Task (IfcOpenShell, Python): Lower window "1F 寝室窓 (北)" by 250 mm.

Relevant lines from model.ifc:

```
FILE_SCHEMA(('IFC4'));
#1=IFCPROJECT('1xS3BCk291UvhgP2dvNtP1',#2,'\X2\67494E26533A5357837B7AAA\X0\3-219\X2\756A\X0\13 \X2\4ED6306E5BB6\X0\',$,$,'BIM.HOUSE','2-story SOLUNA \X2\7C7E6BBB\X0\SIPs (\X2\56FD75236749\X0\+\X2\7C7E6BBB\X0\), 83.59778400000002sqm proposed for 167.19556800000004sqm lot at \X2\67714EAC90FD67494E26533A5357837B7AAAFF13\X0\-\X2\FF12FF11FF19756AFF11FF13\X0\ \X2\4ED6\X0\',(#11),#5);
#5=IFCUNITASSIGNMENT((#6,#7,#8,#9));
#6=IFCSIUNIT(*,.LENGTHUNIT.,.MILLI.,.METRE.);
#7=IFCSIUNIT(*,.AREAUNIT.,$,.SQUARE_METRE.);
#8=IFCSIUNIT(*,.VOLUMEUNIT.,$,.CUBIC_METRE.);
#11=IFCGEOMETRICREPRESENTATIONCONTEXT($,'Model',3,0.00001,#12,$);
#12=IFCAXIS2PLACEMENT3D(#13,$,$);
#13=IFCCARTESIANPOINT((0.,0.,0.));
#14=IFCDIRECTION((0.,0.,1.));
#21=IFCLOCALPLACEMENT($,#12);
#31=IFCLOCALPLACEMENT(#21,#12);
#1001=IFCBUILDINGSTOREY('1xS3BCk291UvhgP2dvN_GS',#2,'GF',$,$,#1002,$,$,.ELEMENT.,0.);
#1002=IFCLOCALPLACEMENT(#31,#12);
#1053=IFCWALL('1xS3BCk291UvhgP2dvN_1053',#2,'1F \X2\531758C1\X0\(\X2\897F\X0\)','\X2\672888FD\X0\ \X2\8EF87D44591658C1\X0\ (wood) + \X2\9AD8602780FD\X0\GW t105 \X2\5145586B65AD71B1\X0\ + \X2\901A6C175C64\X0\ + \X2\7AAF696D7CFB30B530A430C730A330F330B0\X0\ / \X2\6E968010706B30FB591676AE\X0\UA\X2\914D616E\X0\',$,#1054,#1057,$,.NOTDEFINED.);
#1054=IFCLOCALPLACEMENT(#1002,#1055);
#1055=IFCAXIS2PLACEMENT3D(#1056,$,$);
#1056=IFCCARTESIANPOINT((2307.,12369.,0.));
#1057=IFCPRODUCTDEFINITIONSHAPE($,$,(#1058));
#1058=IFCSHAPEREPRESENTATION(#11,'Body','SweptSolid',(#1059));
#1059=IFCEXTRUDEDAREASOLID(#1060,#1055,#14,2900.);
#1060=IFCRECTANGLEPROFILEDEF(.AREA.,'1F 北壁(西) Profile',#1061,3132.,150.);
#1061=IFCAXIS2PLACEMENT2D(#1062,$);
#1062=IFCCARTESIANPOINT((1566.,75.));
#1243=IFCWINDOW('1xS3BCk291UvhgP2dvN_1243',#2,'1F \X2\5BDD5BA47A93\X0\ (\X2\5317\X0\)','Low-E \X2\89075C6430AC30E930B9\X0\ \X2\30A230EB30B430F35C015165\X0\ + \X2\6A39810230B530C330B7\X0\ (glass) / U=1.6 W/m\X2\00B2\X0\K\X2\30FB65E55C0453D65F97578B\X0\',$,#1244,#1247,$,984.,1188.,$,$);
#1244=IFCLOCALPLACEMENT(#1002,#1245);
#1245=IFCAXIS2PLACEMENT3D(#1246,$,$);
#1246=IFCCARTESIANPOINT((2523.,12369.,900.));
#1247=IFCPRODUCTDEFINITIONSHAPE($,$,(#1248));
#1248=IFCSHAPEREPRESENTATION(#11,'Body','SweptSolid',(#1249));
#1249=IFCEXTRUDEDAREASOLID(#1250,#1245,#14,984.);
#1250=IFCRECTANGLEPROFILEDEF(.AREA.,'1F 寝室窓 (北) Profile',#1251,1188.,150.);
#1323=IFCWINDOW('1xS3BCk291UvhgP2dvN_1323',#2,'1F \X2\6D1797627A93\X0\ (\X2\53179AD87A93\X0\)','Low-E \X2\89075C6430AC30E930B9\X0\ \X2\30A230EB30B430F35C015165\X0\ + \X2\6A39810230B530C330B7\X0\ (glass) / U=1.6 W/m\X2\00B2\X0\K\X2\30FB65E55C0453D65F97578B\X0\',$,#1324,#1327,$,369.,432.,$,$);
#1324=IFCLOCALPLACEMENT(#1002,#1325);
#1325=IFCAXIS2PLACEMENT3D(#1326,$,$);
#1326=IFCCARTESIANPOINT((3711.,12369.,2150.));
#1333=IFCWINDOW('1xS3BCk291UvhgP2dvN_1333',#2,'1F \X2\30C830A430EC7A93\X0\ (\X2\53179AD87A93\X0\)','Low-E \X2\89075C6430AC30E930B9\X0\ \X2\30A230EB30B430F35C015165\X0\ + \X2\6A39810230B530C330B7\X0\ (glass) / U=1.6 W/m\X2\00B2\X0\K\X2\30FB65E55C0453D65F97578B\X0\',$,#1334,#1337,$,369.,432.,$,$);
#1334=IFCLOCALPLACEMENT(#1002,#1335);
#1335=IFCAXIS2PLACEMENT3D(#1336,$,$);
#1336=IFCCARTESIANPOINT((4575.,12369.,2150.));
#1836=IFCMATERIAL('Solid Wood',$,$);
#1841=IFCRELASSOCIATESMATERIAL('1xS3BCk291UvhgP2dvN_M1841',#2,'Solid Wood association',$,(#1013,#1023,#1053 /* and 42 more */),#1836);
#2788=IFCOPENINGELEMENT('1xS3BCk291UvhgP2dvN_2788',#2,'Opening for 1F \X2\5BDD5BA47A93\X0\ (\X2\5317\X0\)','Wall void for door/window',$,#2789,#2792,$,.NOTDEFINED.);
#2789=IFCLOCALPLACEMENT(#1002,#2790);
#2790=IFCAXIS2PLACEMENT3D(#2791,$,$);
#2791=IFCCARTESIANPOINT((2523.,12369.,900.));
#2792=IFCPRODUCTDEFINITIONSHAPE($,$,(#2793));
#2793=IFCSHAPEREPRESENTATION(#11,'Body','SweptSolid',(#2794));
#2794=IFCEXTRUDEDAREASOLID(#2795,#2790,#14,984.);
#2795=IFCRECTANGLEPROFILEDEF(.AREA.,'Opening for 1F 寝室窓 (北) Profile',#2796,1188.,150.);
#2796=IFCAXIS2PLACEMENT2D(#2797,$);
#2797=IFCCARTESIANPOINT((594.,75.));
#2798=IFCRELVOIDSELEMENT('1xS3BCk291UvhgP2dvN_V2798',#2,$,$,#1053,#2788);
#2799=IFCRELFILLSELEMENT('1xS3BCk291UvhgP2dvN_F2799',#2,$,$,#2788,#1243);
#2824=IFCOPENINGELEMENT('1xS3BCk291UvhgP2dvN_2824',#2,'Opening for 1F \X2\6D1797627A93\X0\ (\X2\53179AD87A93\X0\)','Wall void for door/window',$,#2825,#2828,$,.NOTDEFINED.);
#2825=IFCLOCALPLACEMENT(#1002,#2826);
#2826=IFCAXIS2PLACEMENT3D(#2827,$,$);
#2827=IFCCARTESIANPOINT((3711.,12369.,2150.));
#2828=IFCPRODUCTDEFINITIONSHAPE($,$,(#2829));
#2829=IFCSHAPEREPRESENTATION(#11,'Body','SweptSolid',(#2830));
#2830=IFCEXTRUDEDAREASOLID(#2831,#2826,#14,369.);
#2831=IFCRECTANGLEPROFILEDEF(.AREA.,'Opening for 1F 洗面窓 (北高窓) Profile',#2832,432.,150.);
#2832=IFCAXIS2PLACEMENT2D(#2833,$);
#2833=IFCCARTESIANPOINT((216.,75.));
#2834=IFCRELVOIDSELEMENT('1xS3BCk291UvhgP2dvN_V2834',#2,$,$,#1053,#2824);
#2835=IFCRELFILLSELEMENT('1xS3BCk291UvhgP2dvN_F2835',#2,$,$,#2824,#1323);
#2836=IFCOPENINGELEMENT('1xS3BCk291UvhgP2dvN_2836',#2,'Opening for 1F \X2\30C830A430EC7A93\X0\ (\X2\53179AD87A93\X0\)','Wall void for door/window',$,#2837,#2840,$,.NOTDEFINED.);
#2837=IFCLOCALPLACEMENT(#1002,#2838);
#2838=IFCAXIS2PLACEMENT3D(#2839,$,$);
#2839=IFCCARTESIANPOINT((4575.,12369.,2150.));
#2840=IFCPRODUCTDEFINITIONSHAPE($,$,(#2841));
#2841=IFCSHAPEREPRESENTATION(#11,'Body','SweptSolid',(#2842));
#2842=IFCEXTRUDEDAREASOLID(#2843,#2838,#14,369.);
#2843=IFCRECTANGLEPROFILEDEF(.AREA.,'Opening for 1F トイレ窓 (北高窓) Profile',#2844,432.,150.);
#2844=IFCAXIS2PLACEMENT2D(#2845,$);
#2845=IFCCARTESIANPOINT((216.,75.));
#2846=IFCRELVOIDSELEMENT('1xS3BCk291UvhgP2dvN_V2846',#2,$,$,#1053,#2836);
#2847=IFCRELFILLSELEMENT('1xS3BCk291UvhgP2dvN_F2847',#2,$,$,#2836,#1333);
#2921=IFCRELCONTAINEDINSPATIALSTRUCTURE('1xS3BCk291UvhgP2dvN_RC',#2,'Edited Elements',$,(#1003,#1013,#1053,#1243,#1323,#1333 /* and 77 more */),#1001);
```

```python
import numpy as np
import ifcopenshell
import ifcopenshell.api.geometry
import ifcopenshell.util.placement
import ifcopenshell.util.unit

model = ifcopenshell.open("model.ifc")
unit_scale = ifcopenshell.util.unit.calculate_unit_scale(model)

window = model.by_guid("1xS3BCk291UvhgP2dvN_1243")
opening = window.FillsVoids[0].RelatingOpeningElement
dz = -0.25 / unit_scale

shift = np.array([0.0, 0.0, dz])
# The window is not placed relative to its opening, so move both.
for product in (opening, window):
    matrix = ifcopenshell.util.placement.get_local_placement(product.ObjectPlacement)
    matrix[:3, 3] += shift
    ifcopenshell.api.geometry.edit_object_placement(model, product=product, matrix=matrix, is_si=False)

print(f"moved by {dz * unit_scale:+.3f} m")

model.write("model_rev.ifc")
```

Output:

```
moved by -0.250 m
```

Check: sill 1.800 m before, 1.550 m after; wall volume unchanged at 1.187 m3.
